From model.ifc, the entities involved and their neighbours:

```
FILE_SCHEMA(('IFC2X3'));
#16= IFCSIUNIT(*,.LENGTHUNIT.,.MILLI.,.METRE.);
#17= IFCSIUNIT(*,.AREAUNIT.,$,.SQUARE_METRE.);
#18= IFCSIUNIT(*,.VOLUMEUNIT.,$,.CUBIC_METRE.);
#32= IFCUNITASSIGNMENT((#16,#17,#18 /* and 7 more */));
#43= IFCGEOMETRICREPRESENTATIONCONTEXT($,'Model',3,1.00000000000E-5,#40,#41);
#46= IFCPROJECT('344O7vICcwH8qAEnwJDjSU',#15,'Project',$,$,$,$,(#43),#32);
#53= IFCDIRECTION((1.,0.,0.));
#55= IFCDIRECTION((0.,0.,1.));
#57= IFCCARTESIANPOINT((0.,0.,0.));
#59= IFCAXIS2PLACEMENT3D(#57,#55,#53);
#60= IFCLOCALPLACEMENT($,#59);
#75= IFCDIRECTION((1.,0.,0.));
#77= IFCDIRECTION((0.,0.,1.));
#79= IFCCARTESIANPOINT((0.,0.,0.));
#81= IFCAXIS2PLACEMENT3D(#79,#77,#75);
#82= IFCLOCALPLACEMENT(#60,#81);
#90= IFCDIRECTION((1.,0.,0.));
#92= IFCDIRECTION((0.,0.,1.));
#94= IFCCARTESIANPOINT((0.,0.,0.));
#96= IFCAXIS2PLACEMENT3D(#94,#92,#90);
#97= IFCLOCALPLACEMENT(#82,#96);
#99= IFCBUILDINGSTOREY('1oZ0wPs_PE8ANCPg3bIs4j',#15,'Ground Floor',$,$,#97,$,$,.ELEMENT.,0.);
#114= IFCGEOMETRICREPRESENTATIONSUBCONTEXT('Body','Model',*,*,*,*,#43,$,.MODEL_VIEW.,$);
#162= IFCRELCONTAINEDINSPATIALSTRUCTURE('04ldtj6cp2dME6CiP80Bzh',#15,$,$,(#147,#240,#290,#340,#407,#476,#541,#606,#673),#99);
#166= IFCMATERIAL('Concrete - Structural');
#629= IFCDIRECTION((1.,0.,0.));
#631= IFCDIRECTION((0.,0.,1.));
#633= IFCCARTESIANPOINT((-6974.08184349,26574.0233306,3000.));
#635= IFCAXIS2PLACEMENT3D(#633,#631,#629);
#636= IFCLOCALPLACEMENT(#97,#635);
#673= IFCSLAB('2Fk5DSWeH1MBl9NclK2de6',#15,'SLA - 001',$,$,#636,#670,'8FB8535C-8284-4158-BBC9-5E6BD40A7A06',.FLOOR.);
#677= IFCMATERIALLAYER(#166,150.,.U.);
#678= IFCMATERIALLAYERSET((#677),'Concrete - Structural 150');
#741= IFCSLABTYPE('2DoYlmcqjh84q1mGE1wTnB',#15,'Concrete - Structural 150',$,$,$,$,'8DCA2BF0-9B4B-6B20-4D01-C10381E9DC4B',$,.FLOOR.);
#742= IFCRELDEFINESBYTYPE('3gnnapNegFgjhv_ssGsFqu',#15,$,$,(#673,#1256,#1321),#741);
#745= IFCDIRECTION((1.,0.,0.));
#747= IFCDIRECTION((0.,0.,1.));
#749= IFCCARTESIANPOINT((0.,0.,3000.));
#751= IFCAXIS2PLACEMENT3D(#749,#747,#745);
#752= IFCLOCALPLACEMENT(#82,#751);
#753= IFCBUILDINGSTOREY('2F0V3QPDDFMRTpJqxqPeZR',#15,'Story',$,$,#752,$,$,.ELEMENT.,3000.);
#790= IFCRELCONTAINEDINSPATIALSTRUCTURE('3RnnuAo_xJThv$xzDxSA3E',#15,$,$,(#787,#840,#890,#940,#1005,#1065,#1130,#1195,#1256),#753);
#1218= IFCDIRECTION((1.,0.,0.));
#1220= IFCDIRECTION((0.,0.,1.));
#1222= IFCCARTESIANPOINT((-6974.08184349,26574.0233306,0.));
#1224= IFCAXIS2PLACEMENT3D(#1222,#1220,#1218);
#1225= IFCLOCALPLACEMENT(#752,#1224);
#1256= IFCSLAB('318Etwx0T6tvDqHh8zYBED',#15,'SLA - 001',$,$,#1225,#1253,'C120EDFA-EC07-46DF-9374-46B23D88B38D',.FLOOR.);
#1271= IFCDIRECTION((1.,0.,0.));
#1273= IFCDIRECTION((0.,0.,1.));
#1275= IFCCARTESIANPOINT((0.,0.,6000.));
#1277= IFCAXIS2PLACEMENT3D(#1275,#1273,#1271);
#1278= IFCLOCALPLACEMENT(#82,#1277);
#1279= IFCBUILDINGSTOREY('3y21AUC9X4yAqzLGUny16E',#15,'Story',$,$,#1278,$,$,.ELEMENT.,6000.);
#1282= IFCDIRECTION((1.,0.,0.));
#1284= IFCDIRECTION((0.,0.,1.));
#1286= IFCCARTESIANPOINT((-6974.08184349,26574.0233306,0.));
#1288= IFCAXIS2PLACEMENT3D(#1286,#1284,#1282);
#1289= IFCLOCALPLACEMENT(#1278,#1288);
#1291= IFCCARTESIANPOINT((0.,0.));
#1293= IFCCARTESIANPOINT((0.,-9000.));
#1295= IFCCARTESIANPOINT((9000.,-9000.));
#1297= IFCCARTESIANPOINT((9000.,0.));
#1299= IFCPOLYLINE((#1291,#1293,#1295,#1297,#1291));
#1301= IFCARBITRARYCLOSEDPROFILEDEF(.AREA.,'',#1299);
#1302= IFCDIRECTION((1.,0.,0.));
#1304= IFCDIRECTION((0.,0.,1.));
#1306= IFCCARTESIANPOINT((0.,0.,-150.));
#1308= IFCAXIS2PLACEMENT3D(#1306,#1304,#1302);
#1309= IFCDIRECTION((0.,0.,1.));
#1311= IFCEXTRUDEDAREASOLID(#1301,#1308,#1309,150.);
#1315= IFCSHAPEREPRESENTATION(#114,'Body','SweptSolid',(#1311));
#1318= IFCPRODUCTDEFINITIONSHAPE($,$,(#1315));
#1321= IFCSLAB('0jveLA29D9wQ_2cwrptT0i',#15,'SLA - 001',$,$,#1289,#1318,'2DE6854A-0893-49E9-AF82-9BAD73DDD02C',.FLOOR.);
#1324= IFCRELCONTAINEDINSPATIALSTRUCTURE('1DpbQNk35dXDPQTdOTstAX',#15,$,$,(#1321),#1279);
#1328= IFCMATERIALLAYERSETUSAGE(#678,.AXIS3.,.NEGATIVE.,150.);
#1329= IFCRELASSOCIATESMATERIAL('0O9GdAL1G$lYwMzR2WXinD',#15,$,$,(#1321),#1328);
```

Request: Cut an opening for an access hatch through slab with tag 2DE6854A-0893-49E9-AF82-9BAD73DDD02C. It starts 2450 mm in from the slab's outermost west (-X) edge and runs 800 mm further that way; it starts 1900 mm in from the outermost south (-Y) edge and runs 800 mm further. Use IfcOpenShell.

```python
import numpy as np
import ifcopenshell
import ifcopenshell.api.feature
import ifcopenshell.api.geometry
import ifcopenshell.api.root
import ifcopenshell.geom
import ifcopenshell.util.placement
import ifcopenshell.util.representation
import ifcopenshell.util.shape
import ifcopenshell.util.unit

model = ifcopenshell.open("model.ifc")
unit_scale = ifcopenshell.util.unit.calculate_unit_scale(model)
settings = ifcopenshell.geom.settings()


def volume(element):
    """Net volume in cubic metres, openings subtracted."""
    shape = ifcopenshell.geom.create_shape(settings, element)
    return ifcopenshell.util.shape.get_volume(shape.geometry)


slab = model.by_guid("0jveLA29D9wQ_2cwrptT0i")
before = volume(slab)

# Extent in the slab's own axes, in metres. The edges named are its -X and -Y sides.
slab_shape = ifcopenshell.geom.create_shape(settings, slab)
vertices = ifcopenshell.util.shape.get_vertices(slab_shape.geometry)
x_min, y_min, bottom = vertices.min(axis=0)
top = vertices[:, 2].max()

opening = ifcopenshell.api.root.create_entity(model, ifc_class="IfcOpeningElement", name="Access hatch opening")
context = ifcopenshell.util.representation.get_context(model, "Model", "Body", "MODEL_VIEW")
width, depth = 0.8, 0.8
outline = [(0.0, 0.0), (width, 0.0), (width, depth), (0.0, depth), (0.0, 0.0)]
# Overshoot both faces by 50 mm so the cut is clean.
shape = ifcopenshell.api.geometry.add_slab_representation(
    model, context=context, depth=top - bottom + 0.1, polyline=outline
)
ifcopenshell.api.geometry.assign_representation(model, product=opening, representation=shape)

matrix = ifcopenshell.util.placement.get_local_placement(slab.ObjectPlacement)
matrix[:, 3] = matrix @ np.append(np.array([x_min + 2.45, y_min + 1.9, bottom - 0.05]) / unit_scale, 1.0)
ifcopenshell.api.geometry.edit_object_placement(model, product=opening, matrix=matrix, is_si=False)
ifcopenshell.api.feature.add_feature(model, feature=opening, element=slab)

after = volume(slab)

print(f"slab volume {before:.3f} -> {after:.3f} m3")

model.write("model_rev.ifc")
```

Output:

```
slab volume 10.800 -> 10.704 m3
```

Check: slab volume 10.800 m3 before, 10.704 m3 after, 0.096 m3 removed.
